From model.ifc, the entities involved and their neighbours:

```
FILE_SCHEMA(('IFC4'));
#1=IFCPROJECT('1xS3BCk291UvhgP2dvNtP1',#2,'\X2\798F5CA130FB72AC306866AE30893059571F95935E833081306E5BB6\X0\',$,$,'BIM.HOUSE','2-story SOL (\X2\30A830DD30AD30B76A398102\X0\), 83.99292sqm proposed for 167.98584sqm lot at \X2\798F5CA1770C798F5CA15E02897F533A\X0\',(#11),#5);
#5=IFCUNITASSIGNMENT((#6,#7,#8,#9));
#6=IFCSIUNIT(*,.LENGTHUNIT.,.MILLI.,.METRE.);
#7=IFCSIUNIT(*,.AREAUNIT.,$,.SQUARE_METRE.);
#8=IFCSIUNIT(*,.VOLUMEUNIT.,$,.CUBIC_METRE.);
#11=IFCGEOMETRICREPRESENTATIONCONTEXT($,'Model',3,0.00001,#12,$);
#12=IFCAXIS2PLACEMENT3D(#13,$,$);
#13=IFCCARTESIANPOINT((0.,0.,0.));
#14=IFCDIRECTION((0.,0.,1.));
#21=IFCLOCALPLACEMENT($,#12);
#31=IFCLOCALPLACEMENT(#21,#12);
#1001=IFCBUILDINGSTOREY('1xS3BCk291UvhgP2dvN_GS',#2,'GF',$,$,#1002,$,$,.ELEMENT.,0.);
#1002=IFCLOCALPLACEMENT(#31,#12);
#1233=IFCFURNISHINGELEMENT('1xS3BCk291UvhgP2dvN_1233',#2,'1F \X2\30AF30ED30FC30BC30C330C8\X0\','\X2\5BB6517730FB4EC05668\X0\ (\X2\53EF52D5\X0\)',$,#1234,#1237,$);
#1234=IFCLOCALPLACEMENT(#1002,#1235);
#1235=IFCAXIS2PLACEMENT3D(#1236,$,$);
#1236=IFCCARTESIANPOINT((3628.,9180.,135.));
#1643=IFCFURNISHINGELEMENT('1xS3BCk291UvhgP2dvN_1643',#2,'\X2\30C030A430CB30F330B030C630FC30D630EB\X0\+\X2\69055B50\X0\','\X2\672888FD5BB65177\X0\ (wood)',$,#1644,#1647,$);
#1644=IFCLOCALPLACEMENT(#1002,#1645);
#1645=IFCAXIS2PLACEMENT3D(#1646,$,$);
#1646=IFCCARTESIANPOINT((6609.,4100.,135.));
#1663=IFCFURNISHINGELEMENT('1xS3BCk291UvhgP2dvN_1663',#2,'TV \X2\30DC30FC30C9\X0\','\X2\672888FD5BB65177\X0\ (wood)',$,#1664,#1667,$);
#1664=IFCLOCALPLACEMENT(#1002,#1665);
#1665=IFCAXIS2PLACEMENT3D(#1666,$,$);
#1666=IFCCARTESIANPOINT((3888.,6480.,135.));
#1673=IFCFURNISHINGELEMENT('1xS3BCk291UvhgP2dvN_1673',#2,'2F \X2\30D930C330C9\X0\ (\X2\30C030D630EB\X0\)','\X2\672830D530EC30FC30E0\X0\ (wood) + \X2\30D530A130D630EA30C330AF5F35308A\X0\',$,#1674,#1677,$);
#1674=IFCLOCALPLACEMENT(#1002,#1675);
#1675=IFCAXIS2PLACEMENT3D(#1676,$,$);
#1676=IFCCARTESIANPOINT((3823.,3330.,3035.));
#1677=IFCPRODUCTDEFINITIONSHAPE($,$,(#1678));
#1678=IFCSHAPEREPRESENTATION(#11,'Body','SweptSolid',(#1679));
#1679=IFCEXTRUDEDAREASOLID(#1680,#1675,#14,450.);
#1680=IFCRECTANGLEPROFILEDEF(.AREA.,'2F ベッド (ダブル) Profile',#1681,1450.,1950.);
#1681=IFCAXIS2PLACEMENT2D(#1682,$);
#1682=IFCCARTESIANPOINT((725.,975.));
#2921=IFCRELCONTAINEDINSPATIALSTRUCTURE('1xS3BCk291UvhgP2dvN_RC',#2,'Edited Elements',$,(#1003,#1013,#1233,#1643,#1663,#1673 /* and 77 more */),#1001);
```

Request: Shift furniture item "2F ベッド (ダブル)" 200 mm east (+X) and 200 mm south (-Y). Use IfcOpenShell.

```python
import ifcopenshell
import ifcopenshell.api.geometry
import ifcopenshell.util.placement
import ifcopenshell.util.unit

model = ifcopenshell.open("model.ifc")
unit_scale = ifcopenshell.util.unit.calculate_unit_scale(model)

item = model.by_guid("1xS3BCk291UvhgP2dvN_1673")
matrix = ifcopenshell.util.placement.get_local_placement(item.ObjectPlacement)
matrix[0, 3] += 0.2 / unit_scale
matrix[1, 3] -= 0.2 / unit_scale
ifcopenshell.api.geometry.edit_object_placement(model, product=item, matrix=matrix, is_si=False)

print(ifcopenshell.util.placement.get_local_placement(item.ObjectPlacement).round(3) + 0.0)

model.write("model_v2.ifc")
```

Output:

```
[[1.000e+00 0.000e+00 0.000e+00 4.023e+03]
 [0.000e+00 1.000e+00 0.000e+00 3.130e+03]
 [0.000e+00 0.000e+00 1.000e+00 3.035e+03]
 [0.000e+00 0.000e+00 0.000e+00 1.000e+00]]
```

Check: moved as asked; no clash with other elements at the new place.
